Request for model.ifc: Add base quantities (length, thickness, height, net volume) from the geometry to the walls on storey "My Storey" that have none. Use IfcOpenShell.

First a look at what the model holds.

```python
import ifcopenshell
import ifcopenshell.util.element
import ifcopenshell.util.unit

model = ifcopenshell.open("model.ifc")
print(model.schema)
for unit_type in ("LENGTHUNIT", "AREAUNIT", "VOLUMEUNIT"):
    print(unit_type, ifcopenshell.util.unit.calculate_unit_scale(model, unit_type))
storey = next(s for s in model.by_type("IfcBuildingStorey") if s.Name == "My Storey")
walls = [e for e in ifcopenshell.util.element.get_decomposition(storey) if e.is_a("IfcWall")]
for e in sorted(walls, key=lambda e: e.id()):
    print(e.id(), e.is_a(), e.Name, list(ifcopenshell.util.element.get_psets(e, qtos_only=True)), sep=" | ")
```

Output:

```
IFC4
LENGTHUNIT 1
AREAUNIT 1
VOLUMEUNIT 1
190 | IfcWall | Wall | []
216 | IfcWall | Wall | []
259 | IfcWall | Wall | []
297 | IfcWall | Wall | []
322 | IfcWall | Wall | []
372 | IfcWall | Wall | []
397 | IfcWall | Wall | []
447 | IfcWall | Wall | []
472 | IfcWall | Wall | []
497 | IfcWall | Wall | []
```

```python
import ifcopenshell
import ifcopenshell.api.pset
import ifcopenshell.geom
import ifcopenshell.util.element
import ifcopenshell.util.shape
import ifcopenshell.util.unit

model = ifcopenshell.open("model.ifc")
unit_scale = ifcopenshell.util.unit.calculate_unit_scale(model)
volume_scale = ifcopenshell.util.unit.calculate_unit_scale(model, "VOLUMEUNIT")
settings = ifcopenshell.geom.settings()

storey = next(s for s in model.by_type("IfcBuildingStorey") if s.Name == "My Storey")
walls = [e for e in ifcopenshell.util.element.get_decomposition(storey) if e.is_a("IfcWall")]

for e in sorted(walls, key=lambda e: e.id()):
    if ifcopenshell.util.element.get_psets(e, qtos_only=True, should_inherit=False):
        continue
    # Geometry comes back in metres, in the element's own axes.
    shape = ifcopenshell.geom.create_shape(settings, e)
    values = {
        "Length": ifcopenshell.util.shape.get_x(shape.geometry) / unit_scale,
        "Width": ifcopenshell.util.shape.get_y(shape.geometry) / unit_scale,
        "Height": ifcopenshell.util.shape.get_z(shape.geometry) / unit_scale,
        "NetVolume": ifcopenshell.util.shape.get_volume(shape.geometry) / volume_scale,
    }
    qto = ifcopenshell.api.pset.add_qto(model, product=e, name="Qto_WallBaseQuantities")
    ifcopenshell.api.pset.edit_qto(model, qto=qto, properties=values)
    print(e.id(), {k: round(v, 3) for k, v in values.items()})

model.write("model_updated.ifc")
```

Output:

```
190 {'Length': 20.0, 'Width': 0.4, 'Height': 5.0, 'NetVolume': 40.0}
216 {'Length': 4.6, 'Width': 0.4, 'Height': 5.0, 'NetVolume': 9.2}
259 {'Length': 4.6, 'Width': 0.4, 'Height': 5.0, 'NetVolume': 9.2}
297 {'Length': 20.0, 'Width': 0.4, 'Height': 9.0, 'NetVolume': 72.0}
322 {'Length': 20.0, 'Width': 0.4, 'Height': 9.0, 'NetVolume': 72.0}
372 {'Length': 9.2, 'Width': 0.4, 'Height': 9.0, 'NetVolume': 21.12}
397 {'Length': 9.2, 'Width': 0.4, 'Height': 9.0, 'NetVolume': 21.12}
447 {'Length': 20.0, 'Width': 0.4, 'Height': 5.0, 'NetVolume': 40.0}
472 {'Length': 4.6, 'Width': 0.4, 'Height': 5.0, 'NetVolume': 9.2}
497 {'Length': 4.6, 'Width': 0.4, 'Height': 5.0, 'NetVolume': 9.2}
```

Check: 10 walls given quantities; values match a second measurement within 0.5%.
